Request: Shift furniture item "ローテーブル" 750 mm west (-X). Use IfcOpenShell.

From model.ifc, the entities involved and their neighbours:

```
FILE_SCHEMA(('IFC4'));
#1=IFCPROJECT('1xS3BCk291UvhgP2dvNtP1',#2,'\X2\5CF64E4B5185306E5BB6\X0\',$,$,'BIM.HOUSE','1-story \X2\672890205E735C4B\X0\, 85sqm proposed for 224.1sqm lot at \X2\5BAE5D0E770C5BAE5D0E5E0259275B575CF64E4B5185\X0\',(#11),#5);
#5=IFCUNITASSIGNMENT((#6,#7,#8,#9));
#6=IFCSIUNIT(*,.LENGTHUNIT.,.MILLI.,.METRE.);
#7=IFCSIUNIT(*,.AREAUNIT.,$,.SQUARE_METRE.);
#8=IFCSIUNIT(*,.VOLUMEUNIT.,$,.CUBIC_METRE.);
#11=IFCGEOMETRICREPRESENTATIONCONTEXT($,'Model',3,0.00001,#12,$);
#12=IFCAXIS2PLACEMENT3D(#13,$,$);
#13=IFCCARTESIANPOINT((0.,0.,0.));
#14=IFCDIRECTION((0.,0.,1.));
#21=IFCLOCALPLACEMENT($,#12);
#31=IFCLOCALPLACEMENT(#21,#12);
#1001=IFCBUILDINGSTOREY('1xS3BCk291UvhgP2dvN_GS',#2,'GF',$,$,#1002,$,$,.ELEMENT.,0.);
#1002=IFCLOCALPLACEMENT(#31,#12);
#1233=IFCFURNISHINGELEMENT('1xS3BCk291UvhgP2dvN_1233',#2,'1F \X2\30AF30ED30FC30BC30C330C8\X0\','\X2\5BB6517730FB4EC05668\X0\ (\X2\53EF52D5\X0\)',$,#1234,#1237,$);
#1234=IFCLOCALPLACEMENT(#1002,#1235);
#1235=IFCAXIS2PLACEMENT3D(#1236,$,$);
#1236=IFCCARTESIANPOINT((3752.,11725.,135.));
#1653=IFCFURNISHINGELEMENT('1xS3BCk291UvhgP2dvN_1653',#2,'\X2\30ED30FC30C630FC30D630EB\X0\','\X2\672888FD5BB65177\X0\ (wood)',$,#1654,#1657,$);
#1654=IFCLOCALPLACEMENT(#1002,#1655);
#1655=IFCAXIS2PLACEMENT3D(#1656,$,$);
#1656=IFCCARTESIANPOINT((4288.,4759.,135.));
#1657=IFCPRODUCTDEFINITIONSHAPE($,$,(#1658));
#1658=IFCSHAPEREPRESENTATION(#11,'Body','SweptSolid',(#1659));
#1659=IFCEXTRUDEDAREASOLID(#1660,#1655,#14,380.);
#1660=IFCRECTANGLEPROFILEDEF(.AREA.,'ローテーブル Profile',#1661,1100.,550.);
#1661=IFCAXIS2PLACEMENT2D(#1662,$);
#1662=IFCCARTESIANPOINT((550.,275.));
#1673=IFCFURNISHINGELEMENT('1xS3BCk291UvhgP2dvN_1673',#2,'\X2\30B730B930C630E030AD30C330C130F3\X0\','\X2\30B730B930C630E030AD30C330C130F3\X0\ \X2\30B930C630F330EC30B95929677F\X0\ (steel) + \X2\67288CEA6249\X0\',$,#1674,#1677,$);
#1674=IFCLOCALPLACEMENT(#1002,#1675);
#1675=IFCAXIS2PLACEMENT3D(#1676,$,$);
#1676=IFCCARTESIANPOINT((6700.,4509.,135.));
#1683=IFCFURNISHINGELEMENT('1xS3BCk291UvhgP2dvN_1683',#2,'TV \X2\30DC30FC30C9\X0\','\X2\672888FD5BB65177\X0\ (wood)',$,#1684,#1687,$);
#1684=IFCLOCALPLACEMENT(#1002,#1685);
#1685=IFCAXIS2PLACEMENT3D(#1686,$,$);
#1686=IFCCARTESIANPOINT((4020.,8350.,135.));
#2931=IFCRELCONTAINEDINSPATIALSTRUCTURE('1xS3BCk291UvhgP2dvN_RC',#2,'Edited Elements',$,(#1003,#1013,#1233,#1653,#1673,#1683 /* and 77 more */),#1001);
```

```python
import ifcopenshell
import ifcopenshell.api.geometry
import ifcopenshell.util.placement

model = ifcopenshell.open("model.ifc")

item = model.by_id(1653)
matrix = ifcopenshell.util.placement.get_local_placement(item.ObjectPlacement)
matrix[0, 3] -= 750.0
ifcopenshell.api.geometry.edit_object_placement(model, product=item, matrix=matrix, is_si=False)

print(ifcopenshell.util.placement.get_local_placement(item.ObjectPlacement).round(3) + 0.0)

model.write("model_v2.ifc")
```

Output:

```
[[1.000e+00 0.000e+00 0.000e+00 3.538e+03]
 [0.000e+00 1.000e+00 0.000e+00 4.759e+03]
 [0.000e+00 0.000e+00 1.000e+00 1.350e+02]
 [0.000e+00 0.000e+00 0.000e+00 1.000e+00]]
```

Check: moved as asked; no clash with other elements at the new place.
